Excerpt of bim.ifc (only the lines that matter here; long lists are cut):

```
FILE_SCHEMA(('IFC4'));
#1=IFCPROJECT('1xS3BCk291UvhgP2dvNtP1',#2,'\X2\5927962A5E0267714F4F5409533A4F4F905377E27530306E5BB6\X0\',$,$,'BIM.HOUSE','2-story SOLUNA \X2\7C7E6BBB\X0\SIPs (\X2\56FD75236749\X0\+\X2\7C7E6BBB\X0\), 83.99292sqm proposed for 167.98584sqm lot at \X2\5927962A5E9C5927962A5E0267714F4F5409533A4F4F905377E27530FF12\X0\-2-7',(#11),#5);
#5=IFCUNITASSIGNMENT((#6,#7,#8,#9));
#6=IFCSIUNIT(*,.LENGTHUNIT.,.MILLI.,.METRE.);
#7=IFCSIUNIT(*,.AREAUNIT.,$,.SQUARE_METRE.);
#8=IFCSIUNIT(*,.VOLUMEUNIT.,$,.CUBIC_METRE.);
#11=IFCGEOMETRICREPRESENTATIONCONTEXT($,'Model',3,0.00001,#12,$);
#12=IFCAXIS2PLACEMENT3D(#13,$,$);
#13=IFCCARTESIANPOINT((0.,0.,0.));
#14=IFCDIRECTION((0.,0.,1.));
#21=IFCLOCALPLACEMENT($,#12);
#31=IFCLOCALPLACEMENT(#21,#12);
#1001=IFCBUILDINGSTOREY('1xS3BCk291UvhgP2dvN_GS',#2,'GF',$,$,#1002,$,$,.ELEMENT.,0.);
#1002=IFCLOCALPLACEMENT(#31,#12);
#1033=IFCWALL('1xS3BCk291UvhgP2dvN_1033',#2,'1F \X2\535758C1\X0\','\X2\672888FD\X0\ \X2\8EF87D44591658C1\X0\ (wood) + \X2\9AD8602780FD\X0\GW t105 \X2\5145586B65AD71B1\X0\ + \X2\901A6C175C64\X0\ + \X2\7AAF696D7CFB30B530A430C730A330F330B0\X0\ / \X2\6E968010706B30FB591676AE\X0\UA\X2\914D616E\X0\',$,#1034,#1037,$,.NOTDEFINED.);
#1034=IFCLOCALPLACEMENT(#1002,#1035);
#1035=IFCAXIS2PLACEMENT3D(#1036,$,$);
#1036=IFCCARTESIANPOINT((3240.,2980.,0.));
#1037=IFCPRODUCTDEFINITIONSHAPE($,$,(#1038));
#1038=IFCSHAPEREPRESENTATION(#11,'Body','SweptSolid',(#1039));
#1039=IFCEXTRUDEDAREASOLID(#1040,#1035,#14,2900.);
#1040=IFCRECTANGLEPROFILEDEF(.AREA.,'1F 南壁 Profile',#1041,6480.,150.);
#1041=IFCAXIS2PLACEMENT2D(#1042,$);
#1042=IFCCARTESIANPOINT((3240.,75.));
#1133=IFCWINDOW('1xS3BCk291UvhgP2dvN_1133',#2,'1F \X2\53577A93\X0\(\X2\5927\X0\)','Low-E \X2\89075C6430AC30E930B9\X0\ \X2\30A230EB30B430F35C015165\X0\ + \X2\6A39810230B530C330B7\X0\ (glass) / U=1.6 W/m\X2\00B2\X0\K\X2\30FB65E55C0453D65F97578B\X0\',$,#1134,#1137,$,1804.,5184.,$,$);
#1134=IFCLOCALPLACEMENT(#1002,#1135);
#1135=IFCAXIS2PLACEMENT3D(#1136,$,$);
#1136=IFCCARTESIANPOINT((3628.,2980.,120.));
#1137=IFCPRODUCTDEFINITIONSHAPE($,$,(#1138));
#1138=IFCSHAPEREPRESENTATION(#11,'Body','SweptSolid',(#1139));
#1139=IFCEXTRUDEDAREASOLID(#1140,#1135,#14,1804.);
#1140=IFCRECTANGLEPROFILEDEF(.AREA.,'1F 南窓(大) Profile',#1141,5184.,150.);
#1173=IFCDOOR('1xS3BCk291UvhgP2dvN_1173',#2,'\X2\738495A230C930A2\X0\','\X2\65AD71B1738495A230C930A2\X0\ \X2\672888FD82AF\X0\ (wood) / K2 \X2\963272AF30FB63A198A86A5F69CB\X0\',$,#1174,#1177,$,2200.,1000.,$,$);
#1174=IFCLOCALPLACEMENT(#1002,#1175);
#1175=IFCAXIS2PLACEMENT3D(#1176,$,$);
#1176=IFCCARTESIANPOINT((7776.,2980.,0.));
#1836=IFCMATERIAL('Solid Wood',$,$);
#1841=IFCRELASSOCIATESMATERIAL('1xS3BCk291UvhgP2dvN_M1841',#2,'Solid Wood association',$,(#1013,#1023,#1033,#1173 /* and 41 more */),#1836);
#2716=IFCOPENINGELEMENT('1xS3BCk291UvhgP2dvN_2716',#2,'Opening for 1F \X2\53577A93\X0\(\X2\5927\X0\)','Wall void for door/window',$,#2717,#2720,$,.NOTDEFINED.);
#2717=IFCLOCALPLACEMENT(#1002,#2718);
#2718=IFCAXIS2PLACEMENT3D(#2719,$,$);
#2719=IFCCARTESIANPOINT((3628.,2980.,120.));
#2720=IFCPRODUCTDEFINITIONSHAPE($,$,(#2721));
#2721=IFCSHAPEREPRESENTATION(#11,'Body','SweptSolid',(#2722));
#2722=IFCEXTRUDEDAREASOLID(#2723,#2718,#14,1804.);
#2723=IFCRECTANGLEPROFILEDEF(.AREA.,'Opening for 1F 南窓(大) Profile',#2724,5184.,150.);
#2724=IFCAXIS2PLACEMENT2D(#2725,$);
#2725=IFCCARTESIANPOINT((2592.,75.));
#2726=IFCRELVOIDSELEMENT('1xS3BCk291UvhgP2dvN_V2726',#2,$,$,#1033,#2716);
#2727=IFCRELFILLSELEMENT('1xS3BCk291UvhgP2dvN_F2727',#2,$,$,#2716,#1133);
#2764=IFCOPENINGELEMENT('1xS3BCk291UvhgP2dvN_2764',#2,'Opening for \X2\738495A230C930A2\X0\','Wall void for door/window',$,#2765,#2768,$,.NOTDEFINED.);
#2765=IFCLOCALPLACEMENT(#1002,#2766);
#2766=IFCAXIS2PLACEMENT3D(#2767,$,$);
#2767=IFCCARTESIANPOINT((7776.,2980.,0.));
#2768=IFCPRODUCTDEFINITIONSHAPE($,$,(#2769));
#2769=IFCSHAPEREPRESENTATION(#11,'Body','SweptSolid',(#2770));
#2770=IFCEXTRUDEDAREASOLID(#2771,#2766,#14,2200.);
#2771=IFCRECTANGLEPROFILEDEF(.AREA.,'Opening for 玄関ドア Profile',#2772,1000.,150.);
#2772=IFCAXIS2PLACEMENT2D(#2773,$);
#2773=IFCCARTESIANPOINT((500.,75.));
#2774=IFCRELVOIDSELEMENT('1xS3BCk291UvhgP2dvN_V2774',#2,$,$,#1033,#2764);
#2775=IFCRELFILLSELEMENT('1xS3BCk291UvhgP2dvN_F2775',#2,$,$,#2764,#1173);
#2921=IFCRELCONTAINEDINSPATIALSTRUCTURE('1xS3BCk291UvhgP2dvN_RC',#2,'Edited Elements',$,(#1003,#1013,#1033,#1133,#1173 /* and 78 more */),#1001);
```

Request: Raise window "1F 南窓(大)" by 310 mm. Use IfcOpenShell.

```python
import numpy as np
import ifcopenshell
import ifcopenshell.api.geometry
import ifcopenshell.util.placement
import ifcopenshell.util.unit

model = ifcopenshell.open("bim.ifc")
unit_scale = ifcopenshell.util.unit.calculate_unit_scale(model)

window = model.by_guid("1xS3BCk291UvhgP2dvN_1133")
opening = window.FillsVoids[0].RelatingOpeningElement
dz = 0.31 / unit_scale

shift = np.array([0.0, 0.0, dz])
# The window is not placed relative to its opening, so move both.
for product in (opening, window):
    matrix = ifcopenshell.util.placement.get_local_placement(product.ObjectPlacement)
    matrix[:3, 3] += shift
    ifcopenshell.api.geometry.edit_object_placement(model, product=product, matrix=matrix, is_si=False)

print(f"moved by {dz * unit_scale:+.3f} m")

model.write("bim_updated.ifc")
```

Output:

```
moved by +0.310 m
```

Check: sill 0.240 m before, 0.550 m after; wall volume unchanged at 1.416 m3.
